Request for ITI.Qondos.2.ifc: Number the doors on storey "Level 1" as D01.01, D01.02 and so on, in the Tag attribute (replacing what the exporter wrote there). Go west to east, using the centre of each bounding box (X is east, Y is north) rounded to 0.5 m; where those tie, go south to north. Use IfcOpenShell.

First a look at what the model holds.

```python
import ifcopenshell
import ifcopenshell.util.element
import ifcopenshell.util.placement

model = ifcopenshell.open("ITI.Qondos.2.ifc")
print(model.schema)
storey = next(s for s in model.by_type("IfcBuildingStorey") if s.Name == "Level 1")
doors = [e for e in ifcopenshell.util.element.get_decomposition(storey) if e.is_a("IfcDoor")]
for e in sorted(doors, key=lambda e: e.id()):
    origin = ifcopenshell.util.placement.get_local_placement(e.ObjectPlacement)[:3, 3]
    print(e.id(), e.Tag, e.Name, origin.round(2) + 0.0, sep=" | ")
```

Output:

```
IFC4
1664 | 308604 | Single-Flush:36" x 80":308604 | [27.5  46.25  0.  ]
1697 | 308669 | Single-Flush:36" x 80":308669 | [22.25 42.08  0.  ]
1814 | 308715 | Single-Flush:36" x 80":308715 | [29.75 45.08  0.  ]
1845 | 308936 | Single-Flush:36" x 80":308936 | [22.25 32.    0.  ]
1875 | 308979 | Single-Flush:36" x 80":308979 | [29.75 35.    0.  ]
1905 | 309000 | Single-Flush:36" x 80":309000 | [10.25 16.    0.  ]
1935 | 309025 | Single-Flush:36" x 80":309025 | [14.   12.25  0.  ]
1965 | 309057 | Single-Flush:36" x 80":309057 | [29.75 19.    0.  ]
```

```python
import ifcopenshell
import ifcopenshell.geom
import ifcopenshell.util.element
import ifcopenshell.util.shape

model = ifcopenshell.open("ITI.Qondos.2.ifc")
settings = ifcopenshell.geom.settings()
settings.set("use-world-coords", True)


def centre(element):
    shape = ifcopenshell.geom.create_shape(settings, element)
    return ifcopenshell.util.shape.get_bbox_centroid(shape.geometry)


storey = next(s for s in model.by_type("IfcBuildingStorey") if s.Name == "Level 1")
doors = [e for e in ifcopenshell.util.element.get_decomposition(storey) if e.is_a("IfcDoor")]

# Insertion points can sit at a corner or the storey origin, so sort by the geometry (in metres).
centres = {e: centre(e) for e in doors}
doors.sort(key=lambda e: (round(centres[e][0] / 0.5), centres[e][1]))

for i, e in enumerate(doors, start=1):
    number = f"D01.{i:02d}"
    e.Tag = number
    print(e.id(), number)

model.write("ITI.Qondos.2_v2.ifc")
```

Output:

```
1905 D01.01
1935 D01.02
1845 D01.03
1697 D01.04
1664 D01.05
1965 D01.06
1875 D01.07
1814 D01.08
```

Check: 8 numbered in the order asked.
